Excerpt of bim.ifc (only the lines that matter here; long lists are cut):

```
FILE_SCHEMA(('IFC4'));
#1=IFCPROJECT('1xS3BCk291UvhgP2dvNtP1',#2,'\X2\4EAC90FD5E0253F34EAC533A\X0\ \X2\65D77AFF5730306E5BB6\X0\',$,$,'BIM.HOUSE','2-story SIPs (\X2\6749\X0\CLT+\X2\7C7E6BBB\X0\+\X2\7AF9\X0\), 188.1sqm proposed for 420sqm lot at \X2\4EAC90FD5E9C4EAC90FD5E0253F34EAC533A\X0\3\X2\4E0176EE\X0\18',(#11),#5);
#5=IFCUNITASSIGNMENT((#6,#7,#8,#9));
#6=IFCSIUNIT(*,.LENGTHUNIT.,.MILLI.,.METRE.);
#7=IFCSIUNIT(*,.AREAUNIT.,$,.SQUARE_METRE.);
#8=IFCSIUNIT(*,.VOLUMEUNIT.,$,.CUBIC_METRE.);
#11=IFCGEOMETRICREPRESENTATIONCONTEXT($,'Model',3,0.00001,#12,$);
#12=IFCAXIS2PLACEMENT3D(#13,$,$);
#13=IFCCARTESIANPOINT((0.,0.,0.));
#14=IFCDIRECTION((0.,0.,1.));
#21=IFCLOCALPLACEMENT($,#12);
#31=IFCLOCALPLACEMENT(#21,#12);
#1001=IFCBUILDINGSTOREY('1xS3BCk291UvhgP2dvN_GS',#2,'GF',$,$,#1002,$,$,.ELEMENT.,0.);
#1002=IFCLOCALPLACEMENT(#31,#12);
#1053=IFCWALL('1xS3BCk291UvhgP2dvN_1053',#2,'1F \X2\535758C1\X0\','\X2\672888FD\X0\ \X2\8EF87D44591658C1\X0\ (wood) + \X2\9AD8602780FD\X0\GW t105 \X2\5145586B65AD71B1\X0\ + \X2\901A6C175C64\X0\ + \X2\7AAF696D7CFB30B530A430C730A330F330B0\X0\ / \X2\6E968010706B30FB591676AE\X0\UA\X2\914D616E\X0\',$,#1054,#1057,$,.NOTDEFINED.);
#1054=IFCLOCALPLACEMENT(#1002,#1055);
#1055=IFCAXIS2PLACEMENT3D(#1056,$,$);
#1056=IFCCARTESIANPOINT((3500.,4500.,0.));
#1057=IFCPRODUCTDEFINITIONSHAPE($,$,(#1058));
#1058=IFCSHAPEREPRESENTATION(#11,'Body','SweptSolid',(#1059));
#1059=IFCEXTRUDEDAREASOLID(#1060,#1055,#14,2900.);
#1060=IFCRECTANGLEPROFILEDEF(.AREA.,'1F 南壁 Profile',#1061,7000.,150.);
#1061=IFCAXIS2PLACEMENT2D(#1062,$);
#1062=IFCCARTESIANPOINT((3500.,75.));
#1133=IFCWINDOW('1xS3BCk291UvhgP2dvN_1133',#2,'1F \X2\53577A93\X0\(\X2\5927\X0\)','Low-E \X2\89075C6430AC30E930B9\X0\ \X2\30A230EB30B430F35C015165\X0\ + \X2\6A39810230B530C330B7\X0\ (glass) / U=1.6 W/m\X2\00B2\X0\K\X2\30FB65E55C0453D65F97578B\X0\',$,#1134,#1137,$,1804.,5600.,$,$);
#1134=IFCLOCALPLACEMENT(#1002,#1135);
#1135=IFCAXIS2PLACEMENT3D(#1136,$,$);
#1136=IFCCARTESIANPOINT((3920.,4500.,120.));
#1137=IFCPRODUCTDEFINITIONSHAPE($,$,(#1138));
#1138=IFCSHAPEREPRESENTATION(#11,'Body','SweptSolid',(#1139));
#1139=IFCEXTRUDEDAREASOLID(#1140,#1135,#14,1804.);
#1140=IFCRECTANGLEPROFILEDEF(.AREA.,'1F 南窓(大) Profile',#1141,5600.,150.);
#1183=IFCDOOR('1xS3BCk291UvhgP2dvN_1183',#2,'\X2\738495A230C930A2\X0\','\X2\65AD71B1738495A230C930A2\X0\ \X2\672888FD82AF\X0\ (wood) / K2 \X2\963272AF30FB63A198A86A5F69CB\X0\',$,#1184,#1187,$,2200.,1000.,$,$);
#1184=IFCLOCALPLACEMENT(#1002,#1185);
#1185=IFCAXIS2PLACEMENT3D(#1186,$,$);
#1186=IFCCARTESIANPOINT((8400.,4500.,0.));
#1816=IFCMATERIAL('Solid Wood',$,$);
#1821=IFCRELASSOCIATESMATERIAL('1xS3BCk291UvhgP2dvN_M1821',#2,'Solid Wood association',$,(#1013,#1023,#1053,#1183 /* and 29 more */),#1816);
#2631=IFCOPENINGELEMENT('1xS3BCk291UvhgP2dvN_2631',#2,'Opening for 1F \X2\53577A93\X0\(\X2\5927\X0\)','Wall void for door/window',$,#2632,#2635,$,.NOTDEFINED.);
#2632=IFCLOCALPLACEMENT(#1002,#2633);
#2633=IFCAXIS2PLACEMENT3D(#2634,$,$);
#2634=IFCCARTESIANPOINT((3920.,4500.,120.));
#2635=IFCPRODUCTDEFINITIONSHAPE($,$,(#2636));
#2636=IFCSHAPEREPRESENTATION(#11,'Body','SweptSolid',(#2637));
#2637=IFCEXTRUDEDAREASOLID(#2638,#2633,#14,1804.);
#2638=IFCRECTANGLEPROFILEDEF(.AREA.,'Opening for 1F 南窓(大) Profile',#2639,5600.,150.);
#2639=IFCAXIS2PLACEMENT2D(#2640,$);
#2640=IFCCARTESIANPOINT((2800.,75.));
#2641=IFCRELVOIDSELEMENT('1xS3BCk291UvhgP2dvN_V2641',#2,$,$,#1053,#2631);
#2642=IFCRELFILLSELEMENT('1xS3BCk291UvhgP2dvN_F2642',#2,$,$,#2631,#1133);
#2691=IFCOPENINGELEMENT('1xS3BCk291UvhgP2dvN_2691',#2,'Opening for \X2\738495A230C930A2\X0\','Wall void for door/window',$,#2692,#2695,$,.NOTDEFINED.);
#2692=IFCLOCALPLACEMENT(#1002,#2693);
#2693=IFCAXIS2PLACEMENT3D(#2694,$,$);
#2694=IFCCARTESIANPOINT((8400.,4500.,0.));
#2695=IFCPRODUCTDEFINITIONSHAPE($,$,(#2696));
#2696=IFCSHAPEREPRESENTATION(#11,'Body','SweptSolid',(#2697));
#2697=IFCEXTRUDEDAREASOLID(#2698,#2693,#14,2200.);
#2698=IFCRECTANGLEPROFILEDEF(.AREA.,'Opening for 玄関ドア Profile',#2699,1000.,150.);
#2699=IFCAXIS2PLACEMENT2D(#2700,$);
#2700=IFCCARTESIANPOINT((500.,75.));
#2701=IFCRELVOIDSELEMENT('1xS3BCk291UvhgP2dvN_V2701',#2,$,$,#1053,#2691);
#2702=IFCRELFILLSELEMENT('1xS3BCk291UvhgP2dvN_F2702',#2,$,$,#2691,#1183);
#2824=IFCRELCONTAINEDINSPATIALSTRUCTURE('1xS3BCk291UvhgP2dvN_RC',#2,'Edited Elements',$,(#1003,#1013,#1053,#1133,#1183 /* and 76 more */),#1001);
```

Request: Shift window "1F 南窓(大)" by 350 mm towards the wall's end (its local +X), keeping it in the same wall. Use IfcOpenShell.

```python
import ifcopenshell
import ifcopenshell.api.geometry
import ifcopenshell.util.placement
import ifcopenshell.util.unit

model = ifcopenshell.open("bim.ifc")
unit_scale = ifcopenshell.util.unit.calculate_unit_scale(model)

window = model.by_guid("1xS3BCk291UvhgP2dvN_1133")
opening = window.FillsVoids[0].RelatingOpeningElement
wall = opening.VoidsElements[0].RelatingBuildingElement

wall_matrix = ifcopenshell.util.placement.get_local_placement(wall.ObjectPlacement)
shift = wall_matrix[:3, 0] * 0.35 / unit_scale
before = ifcopenshell.util.placement.get_local_placement(window.ObjectPlacement)[:3, 3].copy()

# The window is not placed relative to its opening, so move both.
for product in (opening, window):
    matrix = ifcopenshell.util.placement.get_local_placement(product.ObjectPlacement)
    matrix[:3, 3] += shift
    ifcopenshell.api.geometry.edit_object_placement(model, product=product, matrix=matrix, is_si=False)

after = ifcopenshell.util.placement.get_local_placement(window.ObjectPlacement)[:3, 3]
print("window moved by", (after - before).round(3) + 0.0)

model.write("bim-out.ifc")
```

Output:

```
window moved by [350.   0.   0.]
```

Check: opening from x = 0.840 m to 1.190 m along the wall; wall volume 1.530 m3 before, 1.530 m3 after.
